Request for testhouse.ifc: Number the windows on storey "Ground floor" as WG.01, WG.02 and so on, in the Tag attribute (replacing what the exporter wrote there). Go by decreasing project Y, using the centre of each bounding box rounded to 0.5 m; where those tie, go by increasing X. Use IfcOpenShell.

First a look at what the model holds.

```python
import ifcopenshell
import ifcopenshell.util.element
import ifcopenshell.util.placement

model = ifcopenshell.open("testhouse.ifc")
print(model.schema)
storey = next(s for s in model.by_type("IfcBuildingStorey") if s.Name == "Ground floor")
windows = [e for e in ifcopenshell.util.element.get_decomposition(storey) if e.is_a("IfcWindow")]
for e in sorted(windows, key=lambda e: e.id()):
    origin = ifcopenshell.util.placement.get_local_placement(e.ObjectPlacement)[:3, 3]
    print(e.id(), e.Tag, e.Name, origin.round(2) + 0.0, sep=" | ")
```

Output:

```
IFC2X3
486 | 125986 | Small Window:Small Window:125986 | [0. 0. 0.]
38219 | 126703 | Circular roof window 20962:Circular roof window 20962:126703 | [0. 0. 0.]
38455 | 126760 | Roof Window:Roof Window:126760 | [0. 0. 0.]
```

```python
import ifcopenshell
import ifcopenshell.geom
import ifcopenshell.util.element
import ifcopenshell.util.shape

model = ifcopenshell.open("testhouse.ifc")
settings = ifcopenshell.geom.settings()
settings.set("use-world-coords", True)


def centre(element):
    shape = ifcopenshell.geom.create_shape(settings, element)
    return ifcopenshell.util.shape.get_bbox_centroid(shape.geometry)


storey = next(s for s in model.by_type("IfcBuildingStorey") if s.Name == "Ground floor")
windows = [e for e in ifcopenshell.util.element.get_decomposition(storey) if e.is_a("IfcWindow")]

# Insertion points can sit at a corner or the storey origin, so sort by the geometry (in metres).
centres = {e: centre(e) for e in windows}
windows.sort(key=lambda e: (-round(centres[e][1] / 0.5), centres[e][0]))

for i, e in enumerate(windows, start=1):
    number = f"WG.{i:02d}"
    e.Tag = number
    print(e.id(), number)

model.write("testhouse_v2.ifc")
```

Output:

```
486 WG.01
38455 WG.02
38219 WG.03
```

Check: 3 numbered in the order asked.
